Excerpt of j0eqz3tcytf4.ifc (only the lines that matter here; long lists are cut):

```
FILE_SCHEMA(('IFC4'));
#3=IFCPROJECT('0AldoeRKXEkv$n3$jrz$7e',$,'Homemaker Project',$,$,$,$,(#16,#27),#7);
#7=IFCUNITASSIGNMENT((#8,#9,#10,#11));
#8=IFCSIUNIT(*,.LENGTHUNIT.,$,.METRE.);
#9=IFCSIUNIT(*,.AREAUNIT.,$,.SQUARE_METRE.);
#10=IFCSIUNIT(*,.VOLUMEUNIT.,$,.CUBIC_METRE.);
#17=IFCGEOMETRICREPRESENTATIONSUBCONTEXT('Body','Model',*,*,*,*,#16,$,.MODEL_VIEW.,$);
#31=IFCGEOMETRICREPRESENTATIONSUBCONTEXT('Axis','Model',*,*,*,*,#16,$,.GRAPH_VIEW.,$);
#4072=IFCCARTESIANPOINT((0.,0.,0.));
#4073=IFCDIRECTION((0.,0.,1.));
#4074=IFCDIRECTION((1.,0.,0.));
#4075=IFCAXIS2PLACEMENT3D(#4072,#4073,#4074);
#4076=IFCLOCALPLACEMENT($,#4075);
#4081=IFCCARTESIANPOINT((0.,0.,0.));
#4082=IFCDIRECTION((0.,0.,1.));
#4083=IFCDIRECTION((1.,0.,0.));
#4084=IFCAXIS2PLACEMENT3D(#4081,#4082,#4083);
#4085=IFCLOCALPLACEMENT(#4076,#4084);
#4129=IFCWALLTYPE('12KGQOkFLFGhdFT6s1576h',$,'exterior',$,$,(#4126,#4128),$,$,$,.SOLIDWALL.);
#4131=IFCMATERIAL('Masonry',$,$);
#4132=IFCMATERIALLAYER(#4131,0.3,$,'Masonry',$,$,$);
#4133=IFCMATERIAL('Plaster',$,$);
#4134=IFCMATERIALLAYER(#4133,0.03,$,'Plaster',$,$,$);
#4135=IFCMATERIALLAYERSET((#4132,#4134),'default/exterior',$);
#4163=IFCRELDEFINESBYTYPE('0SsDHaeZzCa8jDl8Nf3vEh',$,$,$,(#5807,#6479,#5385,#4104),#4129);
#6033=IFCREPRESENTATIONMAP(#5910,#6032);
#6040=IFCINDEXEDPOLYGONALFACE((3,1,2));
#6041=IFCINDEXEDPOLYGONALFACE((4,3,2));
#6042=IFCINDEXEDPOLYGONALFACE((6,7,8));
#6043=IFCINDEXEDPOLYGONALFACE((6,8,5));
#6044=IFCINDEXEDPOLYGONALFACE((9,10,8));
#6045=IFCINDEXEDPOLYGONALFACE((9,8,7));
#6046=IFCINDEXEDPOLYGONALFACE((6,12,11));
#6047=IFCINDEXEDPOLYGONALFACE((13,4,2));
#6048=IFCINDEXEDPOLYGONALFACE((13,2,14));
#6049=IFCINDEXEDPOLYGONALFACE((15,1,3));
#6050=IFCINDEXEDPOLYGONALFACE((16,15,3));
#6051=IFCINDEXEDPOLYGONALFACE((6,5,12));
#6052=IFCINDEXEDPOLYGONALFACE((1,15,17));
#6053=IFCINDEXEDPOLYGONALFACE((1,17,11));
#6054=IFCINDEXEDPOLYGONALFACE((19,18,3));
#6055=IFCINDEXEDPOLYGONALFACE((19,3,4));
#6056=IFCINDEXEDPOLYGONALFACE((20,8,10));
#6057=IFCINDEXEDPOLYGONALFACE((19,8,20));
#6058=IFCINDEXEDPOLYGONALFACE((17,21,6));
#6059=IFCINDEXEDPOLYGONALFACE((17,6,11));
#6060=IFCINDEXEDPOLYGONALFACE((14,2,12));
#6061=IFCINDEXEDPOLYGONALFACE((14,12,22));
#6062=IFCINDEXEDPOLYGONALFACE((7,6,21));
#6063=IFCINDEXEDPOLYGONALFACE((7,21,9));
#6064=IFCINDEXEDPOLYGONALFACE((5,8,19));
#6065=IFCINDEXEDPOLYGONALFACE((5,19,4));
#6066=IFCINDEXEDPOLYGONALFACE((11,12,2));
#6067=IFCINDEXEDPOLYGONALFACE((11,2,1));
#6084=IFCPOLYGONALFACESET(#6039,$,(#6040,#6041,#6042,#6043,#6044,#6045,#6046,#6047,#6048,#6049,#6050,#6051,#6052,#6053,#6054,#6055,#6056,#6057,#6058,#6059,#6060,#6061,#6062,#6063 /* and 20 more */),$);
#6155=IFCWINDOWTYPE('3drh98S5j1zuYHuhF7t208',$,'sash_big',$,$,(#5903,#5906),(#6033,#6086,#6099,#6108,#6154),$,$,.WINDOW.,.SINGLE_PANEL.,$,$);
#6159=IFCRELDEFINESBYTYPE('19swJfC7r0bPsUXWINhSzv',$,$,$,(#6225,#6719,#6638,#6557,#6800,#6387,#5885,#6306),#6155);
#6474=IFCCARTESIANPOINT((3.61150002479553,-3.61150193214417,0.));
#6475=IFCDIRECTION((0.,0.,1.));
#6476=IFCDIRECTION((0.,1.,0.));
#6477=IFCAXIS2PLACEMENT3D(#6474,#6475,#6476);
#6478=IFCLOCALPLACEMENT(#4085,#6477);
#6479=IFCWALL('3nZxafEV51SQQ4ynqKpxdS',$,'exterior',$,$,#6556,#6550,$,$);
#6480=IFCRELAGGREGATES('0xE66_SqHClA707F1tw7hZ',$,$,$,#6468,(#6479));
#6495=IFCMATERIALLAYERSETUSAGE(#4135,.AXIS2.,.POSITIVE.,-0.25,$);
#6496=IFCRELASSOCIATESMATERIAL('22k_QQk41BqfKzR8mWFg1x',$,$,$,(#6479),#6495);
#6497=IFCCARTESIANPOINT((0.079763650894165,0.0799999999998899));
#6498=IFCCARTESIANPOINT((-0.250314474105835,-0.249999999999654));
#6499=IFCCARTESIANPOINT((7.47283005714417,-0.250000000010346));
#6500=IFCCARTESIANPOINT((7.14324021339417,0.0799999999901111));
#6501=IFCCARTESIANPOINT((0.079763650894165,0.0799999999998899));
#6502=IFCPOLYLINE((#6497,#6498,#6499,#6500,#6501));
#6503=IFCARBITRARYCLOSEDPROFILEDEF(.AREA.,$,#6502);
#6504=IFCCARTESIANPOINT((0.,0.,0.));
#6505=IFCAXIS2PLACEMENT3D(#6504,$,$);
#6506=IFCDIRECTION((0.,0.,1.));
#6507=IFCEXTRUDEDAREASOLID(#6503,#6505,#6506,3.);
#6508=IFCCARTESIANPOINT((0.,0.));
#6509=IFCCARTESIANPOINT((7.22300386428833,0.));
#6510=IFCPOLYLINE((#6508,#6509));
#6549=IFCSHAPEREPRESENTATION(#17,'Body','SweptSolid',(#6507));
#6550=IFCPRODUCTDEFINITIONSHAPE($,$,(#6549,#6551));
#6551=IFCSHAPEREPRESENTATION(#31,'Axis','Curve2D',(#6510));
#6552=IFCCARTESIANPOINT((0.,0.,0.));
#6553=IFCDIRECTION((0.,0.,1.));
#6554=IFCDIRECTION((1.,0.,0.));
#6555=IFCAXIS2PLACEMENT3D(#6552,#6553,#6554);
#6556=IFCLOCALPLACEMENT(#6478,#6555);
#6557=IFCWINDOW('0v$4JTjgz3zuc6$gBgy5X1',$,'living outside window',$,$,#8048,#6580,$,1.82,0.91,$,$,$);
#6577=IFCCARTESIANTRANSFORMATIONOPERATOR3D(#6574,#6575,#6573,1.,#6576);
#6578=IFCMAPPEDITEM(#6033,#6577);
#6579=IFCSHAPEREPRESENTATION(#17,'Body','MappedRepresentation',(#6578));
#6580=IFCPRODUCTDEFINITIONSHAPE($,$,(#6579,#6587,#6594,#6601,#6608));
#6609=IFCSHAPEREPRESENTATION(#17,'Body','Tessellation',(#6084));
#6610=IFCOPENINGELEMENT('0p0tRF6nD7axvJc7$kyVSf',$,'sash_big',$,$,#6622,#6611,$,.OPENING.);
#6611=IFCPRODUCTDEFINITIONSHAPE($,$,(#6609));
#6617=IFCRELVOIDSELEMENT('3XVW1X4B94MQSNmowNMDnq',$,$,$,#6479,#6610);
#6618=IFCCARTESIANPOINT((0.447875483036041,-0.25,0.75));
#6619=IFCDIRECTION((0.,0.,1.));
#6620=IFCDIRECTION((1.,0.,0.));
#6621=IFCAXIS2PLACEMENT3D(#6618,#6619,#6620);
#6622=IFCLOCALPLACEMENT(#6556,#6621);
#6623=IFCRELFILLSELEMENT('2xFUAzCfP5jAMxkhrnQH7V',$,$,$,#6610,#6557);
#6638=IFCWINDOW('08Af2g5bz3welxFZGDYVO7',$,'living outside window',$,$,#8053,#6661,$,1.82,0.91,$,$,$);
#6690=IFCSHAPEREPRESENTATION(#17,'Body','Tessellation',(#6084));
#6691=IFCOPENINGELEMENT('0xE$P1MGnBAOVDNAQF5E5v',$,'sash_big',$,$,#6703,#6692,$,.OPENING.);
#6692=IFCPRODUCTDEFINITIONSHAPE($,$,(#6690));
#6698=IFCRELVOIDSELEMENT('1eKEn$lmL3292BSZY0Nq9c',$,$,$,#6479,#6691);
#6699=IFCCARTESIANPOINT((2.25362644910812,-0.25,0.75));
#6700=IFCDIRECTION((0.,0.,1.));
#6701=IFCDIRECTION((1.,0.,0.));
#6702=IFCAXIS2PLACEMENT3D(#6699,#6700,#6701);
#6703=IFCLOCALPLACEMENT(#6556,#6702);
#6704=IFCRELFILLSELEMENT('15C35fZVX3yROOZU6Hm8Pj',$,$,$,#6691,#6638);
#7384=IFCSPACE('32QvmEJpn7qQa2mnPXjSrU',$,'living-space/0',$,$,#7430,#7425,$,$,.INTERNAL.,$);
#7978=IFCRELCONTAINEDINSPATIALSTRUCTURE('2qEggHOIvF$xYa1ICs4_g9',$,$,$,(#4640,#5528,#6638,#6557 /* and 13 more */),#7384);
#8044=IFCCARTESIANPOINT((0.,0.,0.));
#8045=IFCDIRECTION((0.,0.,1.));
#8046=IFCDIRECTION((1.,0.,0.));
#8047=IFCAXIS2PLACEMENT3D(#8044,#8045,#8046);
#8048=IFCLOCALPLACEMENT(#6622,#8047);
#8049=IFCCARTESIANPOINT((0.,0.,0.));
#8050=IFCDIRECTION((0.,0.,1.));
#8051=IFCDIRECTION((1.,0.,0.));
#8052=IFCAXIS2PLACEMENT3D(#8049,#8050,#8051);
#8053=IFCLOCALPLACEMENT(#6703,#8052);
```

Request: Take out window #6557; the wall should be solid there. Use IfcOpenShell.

```python
import ifcopenshell
import ifcopenshell.api.feature
import ifcopenshell.api.root
import ifcopenshell.geom
import ifcopenshell.util.shape

model = ifcopenshell.open("j0eqz3tcytf4.ifc")
settings = ifcopenshell.geom.settings()


def volume(element):
    """Net volume in cubic metres, openings subtracted."""
    shape = ifcopenshell.geom.create_shape(settings, element)
    return ifcopenshell.util.shape.get_volume(shape.geometry)


window = model.by_id(6557)
opening = window.FillsVoids[0].RelatingOpeningElement
wall = opening.VoidsElements[0].RelatingBuildingElement
before = volume(wall)

ifcopenshell.api.root.remove_product(model, product=window)
ifcopenshell.api.feature.remove_feature(model, feature=opening)

after = volume(wall)

print(f"wall volume {before:.3f} -> {after:.3f} m3")

model.write("j0eqz3tcytf4_rev.ifc")
```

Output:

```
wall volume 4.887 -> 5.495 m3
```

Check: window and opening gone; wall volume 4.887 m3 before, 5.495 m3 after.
